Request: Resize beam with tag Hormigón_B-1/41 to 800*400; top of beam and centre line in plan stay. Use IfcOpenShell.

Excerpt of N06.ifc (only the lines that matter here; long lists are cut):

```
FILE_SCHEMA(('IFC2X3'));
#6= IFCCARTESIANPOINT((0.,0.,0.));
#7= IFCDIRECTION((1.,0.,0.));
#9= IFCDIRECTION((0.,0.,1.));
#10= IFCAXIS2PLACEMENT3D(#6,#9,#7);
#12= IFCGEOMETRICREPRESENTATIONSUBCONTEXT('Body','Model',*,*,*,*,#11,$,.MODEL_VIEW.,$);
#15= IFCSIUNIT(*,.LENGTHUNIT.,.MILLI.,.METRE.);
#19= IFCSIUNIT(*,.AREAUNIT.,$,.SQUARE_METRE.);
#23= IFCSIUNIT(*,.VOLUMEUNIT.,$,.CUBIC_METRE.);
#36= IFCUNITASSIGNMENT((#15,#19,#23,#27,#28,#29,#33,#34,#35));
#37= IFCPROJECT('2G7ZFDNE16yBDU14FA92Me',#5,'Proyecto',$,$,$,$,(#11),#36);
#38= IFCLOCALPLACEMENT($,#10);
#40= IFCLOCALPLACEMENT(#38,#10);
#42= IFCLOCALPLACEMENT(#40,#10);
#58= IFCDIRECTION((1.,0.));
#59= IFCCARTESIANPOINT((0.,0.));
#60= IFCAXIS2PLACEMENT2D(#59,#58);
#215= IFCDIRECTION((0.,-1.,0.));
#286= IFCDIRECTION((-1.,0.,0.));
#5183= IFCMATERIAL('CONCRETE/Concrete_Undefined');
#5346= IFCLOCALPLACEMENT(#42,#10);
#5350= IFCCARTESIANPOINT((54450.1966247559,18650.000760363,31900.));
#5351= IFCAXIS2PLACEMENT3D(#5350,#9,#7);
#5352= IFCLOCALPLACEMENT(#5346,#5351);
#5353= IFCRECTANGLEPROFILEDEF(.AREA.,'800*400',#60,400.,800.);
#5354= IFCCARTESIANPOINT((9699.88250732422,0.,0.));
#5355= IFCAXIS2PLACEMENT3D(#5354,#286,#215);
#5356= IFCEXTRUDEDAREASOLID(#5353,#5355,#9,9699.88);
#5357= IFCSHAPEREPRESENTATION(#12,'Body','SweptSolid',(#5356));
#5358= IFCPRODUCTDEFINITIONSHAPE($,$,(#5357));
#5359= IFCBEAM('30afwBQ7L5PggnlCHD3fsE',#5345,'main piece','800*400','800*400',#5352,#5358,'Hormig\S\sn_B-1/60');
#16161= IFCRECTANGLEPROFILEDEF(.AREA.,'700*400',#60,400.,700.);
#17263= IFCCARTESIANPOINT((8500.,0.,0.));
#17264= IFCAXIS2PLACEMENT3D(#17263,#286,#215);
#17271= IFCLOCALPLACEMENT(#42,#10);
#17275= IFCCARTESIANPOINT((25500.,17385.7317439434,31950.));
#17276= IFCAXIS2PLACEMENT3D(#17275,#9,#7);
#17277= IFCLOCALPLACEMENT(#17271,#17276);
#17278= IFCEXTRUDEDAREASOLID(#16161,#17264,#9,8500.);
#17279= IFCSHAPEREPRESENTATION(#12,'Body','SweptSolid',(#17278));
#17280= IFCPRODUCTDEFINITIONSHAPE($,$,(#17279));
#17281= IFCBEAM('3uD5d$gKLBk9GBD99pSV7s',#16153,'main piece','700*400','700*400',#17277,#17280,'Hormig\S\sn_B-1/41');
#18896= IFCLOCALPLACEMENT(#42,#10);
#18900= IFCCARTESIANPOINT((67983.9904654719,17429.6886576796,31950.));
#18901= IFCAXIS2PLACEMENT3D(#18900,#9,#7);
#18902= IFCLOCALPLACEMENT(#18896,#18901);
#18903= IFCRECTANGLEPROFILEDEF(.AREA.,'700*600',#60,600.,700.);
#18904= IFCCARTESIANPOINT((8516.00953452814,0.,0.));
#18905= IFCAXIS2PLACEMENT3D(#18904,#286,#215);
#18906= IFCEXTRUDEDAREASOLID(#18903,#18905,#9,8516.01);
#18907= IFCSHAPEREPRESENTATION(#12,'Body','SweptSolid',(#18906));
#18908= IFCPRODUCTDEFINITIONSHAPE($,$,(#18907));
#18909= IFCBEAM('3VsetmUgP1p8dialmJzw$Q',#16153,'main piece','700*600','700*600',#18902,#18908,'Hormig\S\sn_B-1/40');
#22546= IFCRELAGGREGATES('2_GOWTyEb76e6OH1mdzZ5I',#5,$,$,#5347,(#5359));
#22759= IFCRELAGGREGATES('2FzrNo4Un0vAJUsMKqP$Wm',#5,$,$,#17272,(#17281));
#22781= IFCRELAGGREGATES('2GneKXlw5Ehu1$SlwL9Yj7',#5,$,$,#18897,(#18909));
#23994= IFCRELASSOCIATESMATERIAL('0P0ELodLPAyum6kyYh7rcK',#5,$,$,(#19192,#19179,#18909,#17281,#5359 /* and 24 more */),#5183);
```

```python
import ifcopenshell
import ifcopenshell.util.element
import ifcopenshell.util.representation

model = ifcopenshell.open("N06.ifc")

member = model.by_id(17281)
source = next(p for p in model.by_type("IfcRectangleProfileDef") if p.ProfileName == "800*400")

body = ifcopenshell.util.representation.get_representation(member, "Model", "Body")
solid = body.Items[0]
old_profile = solid.SweptArea

# Copy the section's sizes but keep this member's own profile position.
profile = ifcopenshell.util.element.copy(model, source)
# Profiles are centred, so shift by half the change in depth to hold the top.
shift = (old_profile.YDim - profile.YDim) / 2
x, y = old_profile.Position.Location.Coordinates
up = (0.0, 1.0)  # upwards, in the solid's own plane
location = model.createIfcCartesianPoint((x + up[0] * shift, y + up[1] * shift))
profile.Position = model.createIfcAxis2Placement2D(location, old_profile.Position.RefDirection)
solid.SweptArea = profile
if not model.get_total_inverses(old_profile):
    ifcopenshell.util.element.remove_deep2(model, old_profile)
member.Description = member.Description.replace("700*400", "800*400")
member.ObjectType = member.ObjectType.replace("700*400", "800*400")

print(solid.SweptArea)

model.write("N06-out.ifc")
```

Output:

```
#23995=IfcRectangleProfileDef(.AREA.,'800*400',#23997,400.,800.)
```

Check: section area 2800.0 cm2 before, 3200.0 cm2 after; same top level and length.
